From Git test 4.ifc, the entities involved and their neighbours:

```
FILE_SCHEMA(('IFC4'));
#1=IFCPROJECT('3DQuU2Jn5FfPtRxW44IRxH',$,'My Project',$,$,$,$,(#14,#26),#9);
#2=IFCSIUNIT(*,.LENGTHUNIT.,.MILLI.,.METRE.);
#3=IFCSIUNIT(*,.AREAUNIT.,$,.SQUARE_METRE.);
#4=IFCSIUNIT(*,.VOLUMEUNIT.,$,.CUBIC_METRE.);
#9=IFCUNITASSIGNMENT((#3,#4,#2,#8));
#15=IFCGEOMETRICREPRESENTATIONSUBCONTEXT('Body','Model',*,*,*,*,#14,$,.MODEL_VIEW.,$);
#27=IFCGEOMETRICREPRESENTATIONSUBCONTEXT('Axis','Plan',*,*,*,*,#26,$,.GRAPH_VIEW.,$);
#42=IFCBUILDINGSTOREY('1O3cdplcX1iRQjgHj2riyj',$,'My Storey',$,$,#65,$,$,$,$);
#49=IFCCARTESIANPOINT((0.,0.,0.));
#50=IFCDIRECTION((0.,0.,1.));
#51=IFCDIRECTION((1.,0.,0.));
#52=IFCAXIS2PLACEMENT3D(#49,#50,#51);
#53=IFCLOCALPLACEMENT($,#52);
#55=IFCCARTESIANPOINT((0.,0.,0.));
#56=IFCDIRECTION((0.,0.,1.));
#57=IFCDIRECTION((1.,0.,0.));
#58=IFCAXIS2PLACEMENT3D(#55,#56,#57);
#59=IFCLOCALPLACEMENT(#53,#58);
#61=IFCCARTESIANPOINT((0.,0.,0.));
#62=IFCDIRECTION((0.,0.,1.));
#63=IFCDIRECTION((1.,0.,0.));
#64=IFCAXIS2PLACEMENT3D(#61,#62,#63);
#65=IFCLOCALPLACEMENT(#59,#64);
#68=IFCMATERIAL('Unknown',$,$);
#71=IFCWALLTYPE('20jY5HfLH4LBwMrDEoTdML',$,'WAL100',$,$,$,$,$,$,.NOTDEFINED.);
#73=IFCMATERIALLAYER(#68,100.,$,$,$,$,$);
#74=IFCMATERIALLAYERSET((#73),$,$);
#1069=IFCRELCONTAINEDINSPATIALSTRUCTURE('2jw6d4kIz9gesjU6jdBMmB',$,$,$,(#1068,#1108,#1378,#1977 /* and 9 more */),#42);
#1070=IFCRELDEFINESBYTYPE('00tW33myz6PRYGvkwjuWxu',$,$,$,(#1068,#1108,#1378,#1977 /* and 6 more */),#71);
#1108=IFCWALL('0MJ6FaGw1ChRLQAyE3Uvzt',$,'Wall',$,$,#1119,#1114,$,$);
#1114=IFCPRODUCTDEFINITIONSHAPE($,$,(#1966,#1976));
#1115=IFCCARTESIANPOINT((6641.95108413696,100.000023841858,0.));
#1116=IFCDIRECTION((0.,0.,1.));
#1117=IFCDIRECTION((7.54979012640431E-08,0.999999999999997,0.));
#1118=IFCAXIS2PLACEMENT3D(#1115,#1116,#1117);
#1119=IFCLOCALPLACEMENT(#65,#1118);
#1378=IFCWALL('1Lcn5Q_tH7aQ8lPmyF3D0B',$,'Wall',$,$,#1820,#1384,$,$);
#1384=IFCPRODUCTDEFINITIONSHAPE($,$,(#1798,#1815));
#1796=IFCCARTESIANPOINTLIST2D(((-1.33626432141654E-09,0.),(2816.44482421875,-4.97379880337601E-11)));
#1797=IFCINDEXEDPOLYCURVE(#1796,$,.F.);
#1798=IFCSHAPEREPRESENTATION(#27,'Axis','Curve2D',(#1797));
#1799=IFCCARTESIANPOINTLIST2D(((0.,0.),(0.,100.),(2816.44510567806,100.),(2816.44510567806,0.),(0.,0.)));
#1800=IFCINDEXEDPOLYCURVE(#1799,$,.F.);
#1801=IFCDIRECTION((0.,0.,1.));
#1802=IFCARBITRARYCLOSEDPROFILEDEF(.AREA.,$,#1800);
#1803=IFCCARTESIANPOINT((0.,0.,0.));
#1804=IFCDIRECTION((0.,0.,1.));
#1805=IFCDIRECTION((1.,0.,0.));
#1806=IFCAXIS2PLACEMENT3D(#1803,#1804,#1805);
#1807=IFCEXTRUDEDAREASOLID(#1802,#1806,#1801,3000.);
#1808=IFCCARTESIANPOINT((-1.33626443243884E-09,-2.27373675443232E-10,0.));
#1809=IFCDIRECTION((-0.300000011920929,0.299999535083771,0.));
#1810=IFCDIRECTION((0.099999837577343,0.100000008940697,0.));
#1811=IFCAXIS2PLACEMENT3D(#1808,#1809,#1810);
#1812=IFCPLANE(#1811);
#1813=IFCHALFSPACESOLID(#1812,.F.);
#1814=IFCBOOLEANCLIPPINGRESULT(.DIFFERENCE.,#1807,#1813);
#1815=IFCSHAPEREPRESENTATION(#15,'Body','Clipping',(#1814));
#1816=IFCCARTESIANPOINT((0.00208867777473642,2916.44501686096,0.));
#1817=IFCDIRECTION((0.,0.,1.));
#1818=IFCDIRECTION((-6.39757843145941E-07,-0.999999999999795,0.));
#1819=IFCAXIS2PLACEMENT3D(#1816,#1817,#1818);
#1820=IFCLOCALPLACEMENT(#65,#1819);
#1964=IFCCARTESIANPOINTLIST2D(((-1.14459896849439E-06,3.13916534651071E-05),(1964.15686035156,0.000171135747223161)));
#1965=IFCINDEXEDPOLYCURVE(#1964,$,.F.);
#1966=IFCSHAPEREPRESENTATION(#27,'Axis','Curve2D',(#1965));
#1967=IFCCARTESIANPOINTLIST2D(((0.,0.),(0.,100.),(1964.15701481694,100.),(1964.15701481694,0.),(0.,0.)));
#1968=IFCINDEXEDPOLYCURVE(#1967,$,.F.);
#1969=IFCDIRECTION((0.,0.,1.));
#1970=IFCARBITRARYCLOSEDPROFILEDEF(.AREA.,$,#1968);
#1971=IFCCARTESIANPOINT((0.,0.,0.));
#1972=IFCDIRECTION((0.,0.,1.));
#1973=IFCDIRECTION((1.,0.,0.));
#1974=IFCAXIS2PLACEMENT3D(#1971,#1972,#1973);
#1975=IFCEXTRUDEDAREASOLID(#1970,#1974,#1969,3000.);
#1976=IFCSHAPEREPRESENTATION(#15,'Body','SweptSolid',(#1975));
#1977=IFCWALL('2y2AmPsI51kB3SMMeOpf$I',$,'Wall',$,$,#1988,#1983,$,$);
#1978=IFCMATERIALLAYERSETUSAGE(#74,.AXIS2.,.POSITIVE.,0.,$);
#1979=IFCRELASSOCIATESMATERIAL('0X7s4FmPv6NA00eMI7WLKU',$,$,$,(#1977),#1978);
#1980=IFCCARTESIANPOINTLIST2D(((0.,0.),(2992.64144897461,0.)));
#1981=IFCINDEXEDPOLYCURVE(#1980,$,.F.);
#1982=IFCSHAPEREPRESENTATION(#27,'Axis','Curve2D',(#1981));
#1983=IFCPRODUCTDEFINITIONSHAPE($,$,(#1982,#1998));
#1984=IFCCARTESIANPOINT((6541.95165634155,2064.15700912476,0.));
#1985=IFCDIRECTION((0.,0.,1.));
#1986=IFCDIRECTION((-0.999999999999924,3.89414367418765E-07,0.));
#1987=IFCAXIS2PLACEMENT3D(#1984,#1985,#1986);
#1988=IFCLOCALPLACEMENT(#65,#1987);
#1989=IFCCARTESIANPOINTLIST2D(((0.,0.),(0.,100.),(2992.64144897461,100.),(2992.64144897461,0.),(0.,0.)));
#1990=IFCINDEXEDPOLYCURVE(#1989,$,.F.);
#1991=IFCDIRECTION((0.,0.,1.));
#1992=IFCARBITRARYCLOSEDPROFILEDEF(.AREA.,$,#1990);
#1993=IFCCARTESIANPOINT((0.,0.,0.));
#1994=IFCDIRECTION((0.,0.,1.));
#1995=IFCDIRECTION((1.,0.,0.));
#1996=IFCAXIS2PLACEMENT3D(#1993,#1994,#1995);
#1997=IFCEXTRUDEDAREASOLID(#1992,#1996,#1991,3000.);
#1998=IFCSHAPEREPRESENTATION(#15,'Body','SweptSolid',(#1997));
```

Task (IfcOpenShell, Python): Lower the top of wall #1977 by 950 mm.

```python
import ifcopenshell
import ifcopenshell.geom
import ifcopenshell.util.representation
import ifcopenshell.util.shape
import ifcopenshell.util.unit

model = ifcopenshell.open("Git test 4.ifc")
unit_scale = ifcopenshell.util.unit.calculate_unit_scale(model)
settings = ifcopenshell.geom.settings()


def volume(element):
    """Net volume in cubic metres, openings subtracted."""
    shape = ifcopenshell.geom.create_shape(settings, element)
    return ifcopenshell.util.shape.get_volume(shape.geometry)


wall = model.by_id(1977)
before = volume(wall)

body = ifcopenshell.util.representation.get_representation(wall, "Model", "Body")
solid = body.Items[0]
old_height = solid.Depth
solid.Depth -= 0.95 / unit_scale
after = volume(wall)

print(f"height {old_height:g} -> {solid.Depth:g}, volume {before:.3f} -> {after:.3f} m3")

model.write("Git test 4_v2.ifc")
```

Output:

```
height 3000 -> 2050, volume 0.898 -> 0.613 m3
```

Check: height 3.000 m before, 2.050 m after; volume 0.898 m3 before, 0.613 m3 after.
